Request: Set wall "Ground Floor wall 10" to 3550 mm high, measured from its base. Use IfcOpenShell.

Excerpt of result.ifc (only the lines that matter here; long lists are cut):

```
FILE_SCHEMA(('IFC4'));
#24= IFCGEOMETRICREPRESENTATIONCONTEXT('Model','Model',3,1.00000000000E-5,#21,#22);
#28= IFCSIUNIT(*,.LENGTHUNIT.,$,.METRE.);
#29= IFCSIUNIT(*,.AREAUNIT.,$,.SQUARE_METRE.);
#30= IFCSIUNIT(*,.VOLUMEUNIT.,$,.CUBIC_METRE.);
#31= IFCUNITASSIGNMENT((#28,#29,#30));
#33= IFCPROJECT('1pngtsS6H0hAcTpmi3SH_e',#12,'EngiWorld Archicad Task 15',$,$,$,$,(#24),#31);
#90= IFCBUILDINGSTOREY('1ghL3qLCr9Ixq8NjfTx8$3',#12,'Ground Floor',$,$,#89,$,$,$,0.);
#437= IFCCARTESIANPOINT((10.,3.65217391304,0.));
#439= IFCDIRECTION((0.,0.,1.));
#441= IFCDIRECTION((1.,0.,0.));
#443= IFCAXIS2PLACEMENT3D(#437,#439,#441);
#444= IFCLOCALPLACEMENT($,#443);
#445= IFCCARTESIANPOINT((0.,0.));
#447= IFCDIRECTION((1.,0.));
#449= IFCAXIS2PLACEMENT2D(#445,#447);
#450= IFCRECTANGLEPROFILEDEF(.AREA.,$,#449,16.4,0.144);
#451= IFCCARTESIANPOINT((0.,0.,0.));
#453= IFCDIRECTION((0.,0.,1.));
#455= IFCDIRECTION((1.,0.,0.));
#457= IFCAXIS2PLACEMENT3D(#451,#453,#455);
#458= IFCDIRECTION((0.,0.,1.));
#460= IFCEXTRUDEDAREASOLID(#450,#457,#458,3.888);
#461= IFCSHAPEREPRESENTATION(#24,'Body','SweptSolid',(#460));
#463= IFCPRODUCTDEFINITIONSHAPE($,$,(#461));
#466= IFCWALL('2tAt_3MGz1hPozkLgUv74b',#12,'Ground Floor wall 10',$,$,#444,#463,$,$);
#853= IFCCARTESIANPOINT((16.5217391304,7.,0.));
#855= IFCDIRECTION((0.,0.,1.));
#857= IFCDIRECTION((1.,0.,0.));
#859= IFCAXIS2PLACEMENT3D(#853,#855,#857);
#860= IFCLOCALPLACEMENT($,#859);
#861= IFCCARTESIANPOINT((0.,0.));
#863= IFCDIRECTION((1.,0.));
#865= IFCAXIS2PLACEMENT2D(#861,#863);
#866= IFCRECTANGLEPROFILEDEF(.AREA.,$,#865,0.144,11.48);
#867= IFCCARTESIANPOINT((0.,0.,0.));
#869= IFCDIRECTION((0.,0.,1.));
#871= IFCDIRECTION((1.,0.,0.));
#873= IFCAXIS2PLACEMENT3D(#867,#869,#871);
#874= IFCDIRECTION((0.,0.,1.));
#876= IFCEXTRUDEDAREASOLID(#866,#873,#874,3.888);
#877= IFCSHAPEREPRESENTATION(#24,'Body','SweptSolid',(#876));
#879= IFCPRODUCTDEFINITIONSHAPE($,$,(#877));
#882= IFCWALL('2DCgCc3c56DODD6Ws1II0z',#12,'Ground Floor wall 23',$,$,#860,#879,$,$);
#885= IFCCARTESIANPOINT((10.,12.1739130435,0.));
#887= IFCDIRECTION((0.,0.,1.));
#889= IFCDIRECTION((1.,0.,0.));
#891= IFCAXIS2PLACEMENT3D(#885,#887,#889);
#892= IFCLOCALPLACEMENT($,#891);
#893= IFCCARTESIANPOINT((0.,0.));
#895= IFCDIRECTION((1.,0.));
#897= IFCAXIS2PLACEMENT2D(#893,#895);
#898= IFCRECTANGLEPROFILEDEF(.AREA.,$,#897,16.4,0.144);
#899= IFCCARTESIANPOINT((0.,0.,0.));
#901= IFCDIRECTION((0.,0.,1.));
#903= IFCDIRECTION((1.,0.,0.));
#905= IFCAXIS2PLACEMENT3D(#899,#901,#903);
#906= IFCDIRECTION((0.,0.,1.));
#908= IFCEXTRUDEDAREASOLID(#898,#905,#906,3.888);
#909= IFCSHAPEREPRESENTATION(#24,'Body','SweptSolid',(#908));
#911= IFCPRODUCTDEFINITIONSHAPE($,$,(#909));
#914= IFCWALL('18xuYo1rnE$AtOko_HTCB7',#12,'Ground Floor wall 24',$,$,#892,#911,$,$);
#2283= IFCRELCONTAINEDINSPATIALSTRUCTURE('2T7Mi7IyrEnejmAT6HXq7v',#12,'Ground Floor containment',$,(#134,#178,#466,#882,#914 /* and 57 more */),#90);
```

```python
import ifcopenshell
import ifcopenshell.geom
import ifcopenshell.util.shape
import ifcopenshell.util.unit

model = ifcopenshell.open("result.ifc")
unit_scale = ifcopenshell.util.unit.calculate_unit_scale(model)
settings = ifcopenshell.geom.settings()


def volume(element):
    """Net volume in cubic metres, openings subtracted."""
    shape = ifcopenshell.geom.create_shape(settings, element)
    return ifcopenshell.util.shape.get_volume(shape.geometry)


wall = model.by_guid("2tAt_3MGz1hPozkLgUv74b")
before = volume(wall)

body = next(r for r in wall.Representation.Representations if r.RepresentationIdentifier == "Body")
solid = body.Items[0]
old_height = solid.Depth
solid.Depth = 3.55 / unit_scale
after = volume(wall)

print(f"height {old_height:g} -> {solid.Depth:g}, volume {before:.3f} -> {after:.3f} m3")

model.write("result-out.ifc")
```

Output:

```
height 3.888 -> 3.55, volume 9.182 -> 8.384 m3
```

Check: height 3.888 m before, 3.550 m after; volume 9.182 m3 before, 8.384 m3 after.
